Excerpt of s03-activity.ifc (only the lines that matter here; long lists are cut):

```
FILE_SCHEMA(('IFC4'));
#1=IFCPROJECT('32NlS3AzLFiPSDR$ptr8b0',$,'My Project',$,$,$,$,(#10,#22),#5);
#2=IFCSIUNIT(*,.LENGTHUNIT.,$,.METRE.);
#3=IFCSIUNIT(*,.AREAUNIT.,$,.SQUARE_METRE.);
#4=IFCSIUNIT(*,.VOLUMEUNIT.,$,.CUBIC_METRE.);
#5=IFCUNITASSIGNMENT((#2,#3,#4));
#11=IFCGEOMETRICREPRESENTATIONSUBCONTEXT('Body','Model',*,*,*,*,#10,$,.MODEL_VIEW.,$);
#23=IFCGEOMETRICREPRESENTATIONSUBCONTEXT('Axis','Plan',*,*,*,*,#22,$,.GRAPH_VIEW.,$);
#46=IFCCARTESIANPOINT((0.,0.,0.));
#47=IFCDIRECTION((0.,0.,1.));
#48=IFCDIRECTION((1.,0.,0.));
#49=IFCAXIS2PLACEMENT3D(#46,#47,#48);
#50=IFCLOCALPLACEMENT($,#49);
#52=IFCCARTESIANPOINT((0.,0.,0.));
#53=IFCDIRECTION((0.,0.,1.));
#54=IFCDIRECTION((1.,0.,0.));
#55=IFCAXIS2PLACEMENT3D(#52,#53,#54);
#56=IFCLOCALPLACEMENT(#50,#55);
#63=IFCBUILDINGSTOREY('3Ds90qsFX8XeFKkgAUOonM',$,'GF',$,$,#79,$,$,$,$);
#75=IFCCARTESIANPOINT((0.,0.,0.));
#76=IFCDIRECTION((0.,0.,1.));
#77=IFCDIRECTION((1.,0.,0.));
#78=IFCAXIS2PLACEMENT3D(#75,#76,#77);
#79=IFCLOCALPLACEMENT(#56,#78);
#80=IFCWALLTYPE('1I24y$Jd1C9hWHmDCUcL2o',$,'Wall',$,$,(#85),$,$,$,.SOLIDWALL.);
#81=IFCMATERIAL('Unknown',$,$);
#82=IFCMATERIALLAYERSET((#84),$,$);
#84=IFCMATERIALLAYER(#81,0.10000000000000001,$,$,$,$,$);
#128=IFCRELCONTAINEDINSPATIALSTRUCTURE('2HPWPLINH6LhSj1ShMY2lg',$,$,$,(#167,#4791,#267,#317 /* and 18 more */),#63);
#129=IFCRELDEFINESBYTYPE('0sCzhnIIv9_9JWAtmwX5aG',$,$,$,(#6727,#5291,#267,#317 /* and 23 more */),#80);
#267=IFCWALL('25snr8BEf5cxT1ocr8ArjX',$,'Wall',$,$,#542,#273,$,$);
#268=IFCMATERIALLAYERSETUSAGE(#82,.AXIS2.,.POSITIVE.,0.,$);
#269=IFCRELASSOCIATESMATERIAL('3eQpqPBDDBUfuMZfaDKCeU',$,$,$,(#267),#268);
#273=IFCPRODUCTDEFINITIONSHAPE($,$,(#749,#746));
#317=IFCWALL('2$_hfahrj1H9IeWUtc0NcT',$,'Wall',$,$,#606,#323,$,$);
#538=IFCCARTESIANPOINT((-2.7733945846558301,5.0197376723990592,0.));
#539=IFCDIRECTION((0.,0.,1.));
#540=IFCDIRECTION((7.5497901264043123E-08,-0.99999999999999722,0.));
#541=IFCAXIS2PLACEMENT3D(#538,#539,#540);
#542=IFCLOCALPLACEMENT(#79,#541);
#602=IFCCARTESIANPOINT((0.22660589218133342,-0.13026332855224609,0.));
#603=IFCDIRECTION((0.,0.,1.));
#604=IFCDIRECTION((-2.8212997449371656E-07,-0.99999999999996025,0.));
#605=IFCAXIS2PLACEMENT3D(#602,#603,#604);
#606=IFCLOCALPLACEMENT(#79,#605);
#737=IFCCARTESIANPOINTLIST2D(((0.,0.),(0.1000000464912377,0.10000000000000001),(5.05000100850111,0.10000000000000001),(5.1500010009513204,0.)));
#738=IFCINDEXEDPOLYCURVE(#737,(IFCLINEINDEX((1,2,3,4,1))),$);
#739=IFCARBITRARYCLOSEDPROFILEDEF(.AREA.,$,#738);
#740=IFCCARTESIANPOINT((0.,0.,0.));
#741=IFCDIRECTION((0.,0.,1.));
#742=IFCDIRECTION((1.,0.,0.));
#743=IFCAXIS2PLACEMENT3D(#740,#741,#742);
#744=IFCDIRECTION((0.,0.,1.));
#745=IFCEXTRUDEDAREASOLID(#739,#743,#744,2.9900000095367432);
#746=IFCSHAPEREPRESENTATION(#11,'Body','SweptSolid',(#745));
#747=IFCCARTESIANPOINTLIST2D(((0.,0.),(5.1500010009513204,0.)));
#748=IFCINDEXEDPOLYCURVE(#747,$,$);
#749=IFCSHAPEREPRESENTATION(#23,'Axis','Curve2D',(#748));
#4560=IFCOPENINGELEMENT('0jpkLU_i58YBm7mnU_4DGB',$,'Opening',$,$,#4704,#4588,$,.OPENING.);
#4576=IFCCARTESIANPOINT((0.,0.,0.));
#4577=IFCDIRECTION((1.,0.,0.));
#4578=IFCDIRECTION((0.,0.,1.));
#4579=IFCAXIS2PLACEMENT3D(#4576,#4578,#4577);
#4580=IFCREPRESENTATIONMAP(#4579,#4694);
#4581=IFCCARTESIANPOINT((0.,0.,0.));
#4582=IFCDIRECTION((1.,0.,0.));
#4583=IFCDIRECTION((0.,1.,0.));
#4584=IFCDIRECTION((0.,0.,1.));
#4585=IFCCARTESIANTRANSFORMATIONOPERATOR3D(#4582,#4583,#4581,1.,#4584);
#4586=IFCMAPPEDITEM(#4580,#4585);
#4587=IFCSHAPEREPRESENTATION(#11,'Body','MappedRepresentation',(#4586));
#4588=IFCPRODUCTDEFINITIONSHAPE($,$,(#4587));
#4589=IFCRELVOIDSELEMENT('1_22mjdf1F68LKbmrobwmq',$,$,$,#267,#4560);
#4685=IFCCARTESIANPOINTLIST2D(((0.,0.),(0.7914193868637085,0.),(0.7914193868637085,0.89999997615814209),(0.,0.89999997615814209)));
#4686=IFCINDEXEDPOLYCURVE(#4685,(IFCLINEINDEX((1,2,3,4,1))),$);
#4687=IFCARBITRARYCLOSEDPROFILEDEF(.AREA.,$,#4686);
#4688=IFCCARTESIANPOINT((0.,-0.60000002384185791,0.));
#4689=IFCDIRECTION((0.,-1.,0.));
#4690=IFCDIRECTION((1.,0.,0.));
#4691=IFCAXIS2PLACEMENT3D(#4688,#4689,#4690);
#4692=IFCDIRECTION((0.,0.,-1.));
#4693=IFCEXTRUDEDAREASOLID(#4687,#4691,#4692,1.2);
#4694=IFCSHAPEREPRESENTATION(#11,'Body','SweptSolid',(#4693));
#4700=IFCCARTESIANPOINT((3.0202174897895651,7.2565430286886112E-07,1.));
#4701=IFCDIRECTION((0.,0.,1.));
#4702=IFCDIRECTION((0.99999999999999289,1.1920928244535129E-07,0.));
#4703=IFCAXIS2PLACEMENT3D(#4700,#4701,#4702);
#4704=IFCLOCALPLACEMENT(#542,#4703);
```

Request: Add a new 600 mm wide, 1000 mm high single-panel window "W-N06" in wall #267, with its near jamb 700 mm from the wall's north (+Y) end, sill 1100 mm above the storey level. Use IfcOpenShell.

```python
import numpy as np
import ifcopenshell
import ifcopenshell.api.feature
import ifcopenshell.api.geometry
import ifcopenshell.api.root
import ifcopenshell.api.spatial
import ifcopenshell.geom
import ifcopenshell.util.element
import ifcopenshell.util.placement
import ifcopenshell.util.representation
import ifcopenshell.util.shape
import ifcopenshell.util.unit

model = ifcopenshell.open("s03-activity.ifc")
unit_scale = ifcopenshell.util.unit.calculate_unit_scale(model)
settings = ifcopenshell.geom.settings()


def volume(element):
    """Net volume in cubic metres, openings subtracted."""
    shape = ifcopenshell.geom.create_shape(settings, element)
    return ifcopenshell.util.shape.get_volume(shape.geometry)


wall = model.by_guid("25snr8BEf5cxT1ocr8ArjX")
storey = ifcopenshell.util.element.get_container(wall, ifc_class="IfcBuildingStorey")
context = ifcopenshell.util.representation.get_context(model, "Model", "Body", "MODEL_VIEW")
before = volume(wall)

width, height, from_end, sill = 0.6, 1, 0.7, 1.1  # metres

# The wall runs along its own X axis, and the end named is its -X end.
wall_shape = ifcopenshell.geom.create_shape(settings, wall)
x, y, z = ifcopenshell.util.shape.get_vertices(wall_shape.geometry).T
start = x.min() + from_end
face, thickness = float(y.min()), float(y.max() - y.min())
wall_matrix = ifcopenshell.util.placement.get_local_placement(wall.ObjectPlacement)
level = ifcopenshell.util.placement.get_local_placement(storey.ObjectPlacement)[2, 3]


def in_wall(x, y):
    """Placement at x, y metres in the wall's axes, at sill height."""
    matrix = wall_matrix.copy()
    matrix[:, 3] = wall_matrix @ np.array([x / unit_scale, y / unit_scale, 0.0, 1.0])
    matrix[2, 3] = level + sill / unit_scale
    return matrix


# Opening: a box that overshoots both wall faces by 50 mm.
opening = ifcopenshell.api.root.create_entity(model, ifc_class="IfcOpeningElement", predefined_type="OPENING")
box = ifcopenshell.api.geometry.add_wall_representation(
    model, context=context, length=width, height=height, thickness=thickness + 0.1
)
ifcopenshell.api.geometry.assign_representation(model, product=opening, representation=box)
ifcopenshell.api.geometry.edit_object_placement(model, product=opening, matrix=in_wall(start, face - 0.05), is_si=False)
ifcopenshell.api.feature.add_feature(model, feature=opening, element=wall)

window = ifcopenshell.api.root.create_entity(model, ifc_class="IfcWindow", name="W-N06", predefined_type="WINDOW")
window.OverallWidth, window.OverallHeight = width / unit_scale, height / unit_scale
window.PartitioningType = "SINGLE_PANEL"
body = ifcopenshell.api.geometry.add_window_representation(
    model,
    context=context,
    overall_width=window.OverallWidth,
    overall_height=window.OverallHeight,
    partition_type="SINGLE_PANEL",
)
ifcopenshell.api.geometry.assign_representation(model, product=window, representation=body)
ifcopenshell.api.spatial.assign_container(model, products=[window], relating_structure=storey)
ifcopenshell.api.feature.add_filling(model, opening=opening, element=window)

# Centre the window in the wall's thickness.
ifcopenshell.api.geometry.edit_object_placement(model, product=window, matrix=in_wall(start, face), is_si=False)
window_shape = ifcopenshell.geom.create_shape(settings, window)
depth = ifcopenshell.util.shape.get_vertices(window_shape.geometry)[:, 1]
offset = face + thickness / 2 - (depth.min() + depth.max()) / 2
ifcopenshell.api.geometry.edit_object_placement(model, product=window, matrix=in_wall(start, offset), is_si=False)

after = volume(wall)

print(f"wall volume {before:.3f} -> {after:.3f} m3")

model.write("s03-activity-out.ifc")
```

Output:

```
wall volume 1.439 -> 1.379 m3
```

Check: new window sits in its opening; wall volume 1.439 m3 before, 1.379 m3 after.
